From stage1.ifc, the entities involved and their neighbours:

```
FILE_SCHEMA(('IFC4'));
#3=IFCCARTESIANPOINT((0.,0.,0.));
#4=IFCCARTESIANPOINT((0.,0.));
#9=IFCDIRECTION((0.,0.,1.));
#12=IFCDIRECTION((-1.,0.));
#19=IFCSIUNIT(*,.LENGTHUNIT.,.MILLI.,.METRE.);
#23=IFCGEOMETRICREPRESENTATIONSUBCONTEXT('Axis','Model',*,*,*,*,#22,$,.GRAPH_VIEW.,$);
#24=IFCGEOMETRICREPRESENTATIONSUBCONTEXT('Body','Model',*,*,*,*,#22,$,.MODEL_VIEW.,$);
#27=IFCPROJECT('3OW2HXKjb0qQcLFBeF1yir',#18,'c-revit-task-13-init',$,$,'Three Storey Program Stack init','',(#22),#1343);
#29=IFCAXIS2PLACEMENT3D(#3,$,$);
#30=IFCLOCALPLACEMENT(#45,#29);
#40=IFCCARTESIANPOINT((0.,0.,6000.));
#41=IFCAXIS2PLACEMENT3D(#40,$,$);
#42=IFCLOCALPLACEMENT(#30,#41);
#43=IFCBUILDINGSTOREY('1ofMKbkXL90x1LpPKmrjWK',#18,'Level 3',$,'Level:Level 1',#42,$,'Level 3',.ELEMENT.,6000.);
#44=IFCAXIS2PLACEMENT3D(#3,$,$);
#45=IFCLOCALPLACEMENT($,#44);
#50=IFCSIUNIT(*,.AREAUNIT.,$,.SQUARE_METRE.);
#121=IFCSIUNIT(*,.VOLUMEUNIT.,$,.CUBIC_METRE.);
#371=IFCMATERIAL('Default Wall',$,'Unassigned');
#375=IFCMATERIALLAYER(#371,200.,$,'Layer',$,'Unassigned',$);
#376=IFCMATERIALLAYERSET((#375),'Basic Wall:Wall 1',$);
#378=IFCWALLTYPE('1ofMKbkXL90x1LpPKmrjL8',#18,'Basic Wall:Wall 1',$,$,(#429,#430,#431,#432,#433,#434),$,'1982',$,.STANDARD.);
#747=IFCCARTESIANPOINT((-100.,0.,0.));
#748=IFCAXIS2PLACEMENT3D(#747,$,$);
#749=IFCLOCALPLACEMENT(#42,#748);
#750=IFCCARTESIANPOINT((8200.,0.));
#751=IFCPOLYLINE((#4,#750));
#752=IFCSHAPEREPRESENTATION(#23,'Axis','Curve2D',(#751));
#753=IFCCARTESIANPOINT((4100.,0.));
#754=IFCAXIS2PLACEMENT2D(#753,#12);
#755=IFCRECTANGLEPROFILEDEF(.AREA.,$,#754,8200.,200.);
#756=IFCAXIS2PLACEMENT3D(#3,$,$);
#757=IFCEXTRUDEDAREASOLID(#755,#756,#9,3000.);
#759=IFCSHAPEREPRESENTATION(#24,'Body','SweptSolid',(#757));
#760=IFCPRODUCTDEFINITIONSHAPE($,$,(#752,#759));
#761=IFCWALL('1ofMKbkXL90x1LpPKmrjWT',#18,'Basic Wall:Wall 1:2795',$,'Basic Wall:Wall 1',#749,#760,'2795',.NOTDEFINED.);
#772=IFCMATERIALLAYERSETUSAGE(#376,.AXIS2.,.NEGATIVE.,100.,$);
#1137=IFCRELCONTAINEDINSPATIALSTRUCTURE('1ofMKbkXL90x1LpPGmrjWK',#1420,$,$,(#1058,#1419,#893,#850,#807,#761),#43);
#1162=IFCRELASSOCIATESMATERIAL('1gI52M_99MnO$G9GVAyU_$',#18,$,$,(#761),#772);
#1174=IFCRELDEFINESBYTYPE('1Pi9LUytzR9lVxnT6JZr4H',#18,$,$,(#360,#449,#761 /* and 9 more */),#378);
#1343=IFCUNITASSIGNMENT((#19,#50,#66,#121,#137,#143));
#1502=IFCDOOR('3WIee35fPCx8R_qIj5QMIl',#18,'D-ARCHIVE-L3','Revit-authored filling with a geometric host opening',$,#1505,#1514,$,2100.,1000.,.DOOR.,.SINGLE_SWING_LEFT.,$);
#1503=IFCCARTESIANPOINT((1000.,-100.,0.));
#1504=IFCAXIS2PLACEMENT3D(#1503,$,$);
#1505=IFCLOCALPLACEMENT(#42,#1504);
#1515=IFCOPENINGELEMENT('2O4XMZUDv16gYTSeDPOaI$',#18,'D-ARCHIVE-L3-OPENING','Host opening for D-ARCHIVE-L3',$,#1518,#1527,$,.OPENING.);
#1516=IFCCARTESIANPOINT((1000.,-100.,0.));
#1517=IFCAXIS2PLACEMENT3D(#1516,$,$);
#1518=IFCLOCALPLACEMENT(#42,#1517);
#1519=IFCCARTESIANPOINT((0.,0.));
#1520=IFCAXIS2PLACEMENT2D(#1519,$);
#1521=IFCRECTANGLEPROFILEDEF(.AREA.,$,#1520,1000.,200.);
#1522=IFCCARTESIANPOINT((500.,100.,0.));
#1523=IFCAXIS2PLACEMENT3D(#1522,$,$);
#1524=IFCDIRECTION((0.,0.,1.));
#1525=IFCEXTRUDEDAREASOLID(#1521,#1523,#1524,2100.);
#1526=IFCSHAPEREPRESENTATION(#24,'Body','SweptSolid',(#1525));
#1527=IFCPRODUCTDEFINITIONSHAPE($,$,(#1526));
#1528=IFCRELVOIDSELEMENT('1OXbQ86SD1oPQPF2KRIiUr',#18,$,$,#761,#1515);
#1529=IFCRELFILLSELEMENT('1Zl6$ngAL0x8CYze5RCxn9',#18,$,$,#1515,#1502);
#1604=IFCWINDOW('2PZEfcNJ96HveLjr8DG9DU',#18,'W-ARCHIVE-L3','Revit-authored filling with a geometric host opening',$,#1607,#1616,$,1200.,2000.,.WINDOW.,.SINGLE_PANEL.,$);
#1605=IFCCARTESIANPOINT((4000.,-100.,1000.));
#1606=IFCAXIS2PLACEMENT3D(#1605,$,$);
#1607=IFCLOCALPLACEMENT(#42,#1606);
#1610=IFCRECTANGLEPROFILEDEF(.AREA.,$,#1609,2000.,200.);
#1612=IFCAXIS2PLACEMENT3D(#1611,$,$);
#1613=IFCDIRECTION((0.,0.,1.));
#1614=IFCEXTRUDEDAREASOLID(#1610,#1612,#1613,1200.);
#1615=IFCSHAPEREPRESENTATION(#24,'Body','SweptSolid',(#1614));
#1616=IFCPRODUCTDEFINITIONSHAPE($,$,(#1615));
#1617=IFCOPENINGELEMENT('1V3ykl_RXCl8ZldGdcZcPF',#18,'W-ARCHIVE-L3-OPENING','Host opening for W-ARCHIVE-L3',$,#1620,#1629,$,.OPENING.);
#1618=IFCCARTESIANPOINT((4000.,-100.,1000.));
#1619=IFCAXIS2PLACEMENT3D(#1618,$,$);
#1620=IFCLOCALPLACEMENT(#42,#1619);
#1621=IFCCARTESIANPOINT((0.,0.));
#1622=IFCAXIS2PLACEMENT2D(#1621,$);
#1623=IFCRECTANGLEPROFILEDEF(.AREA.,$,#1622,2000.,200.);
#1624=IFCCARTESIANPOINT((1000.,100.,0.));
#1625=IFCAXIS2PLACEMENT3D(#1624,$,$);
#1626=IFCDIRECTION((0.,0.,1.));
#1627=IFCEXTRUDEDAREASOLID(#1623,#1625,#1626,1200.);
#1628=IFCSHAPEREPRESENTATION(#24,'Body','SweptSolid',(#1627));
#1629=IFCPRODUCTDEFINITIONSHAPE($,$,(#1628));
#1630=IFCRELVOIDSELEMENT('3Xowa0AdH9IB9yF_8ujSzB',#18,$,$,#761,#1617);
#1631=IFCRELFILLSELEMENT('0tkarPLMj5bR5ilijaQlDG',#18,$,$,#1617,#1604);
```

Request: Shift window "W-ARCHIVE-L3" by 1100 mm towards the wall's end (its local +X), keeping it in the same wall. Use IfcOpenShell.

```python
import ifcopenshell
import ifcopenshell.api.geometry
import ifcopenshell.util.placement

model = ifcopenshell.open("stage1.ifc")

window = model.by_id(1604)
opening = window.FillsVoids[0].RelatingOpeningElement
wall = opening.VoidsElements[0].RelatingBuildingElement

wall_matrix = ifcopenshell.util.placement.get_local_placement(wall.ObjectPlacement)
shift = wall_matrix[:3, 0] * 1100.0
before = ifcopenshell.util.placement.get_local_placement(window.ObjectPlacement)[:3, 3].copy()

# The window is not placed relative to its opening, so move both.
for product in (opening, window):
    matrix = ifcopenshell.util.placement.get_local_placement(product.ObjectPlacement)
    matrix[:3, 3] += shift
    ifcopenshell.api.geometry.edit_object_placement(model, product=product, matrix=matrix, is_si=False)

after = ifcopenshell.util.placement.get_local_placement(window.ObjectPlacement)[:3, 3]
print("window moved by", (after - before).round(3) + 0.0)

model.write("stage1-out.ifc")
```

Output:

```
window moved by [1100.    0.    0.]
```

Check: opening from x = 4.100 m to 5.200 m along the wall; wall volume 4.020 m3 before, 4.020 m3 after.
